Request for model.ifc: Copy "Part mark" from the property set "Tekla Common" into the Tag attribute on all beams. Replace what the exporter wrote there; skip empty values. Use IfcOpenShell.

First a look at what the model holds.

```python
import ifcopenshell
import ifcopenshell.util.element

model = ifcopenshell.open("model.ifc")
print(model.schema)
beams = model.by_type("IfcBeam")
print(len(beams), "beams")
for e in beams[:8]:
    source = ifcopenshell.util.element.get_pset(e, "Tekla Common", "Part mark")
    target = e.Tag
    print(e.id(), repr(source), repr(target), sep=" | ")
```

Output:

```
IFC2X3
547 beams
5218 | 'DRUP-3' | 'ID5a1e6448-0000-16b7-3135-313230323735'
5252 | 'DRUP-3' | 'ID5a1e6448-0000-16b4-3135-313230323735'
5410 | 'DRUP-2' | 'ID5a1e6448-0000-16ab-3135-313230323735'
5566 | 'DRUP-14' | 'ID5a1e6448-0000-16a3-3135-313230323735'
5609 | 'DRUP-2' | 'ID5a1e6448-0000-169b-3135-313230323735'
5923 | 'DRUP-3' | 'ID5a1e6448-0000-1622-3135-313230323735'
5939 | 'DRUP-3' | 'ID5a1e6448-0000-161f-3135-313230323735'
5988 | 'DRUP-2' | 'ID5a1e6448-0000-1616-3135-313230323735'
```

```python
import ifcopenshell
import ifcopenshell.util.element

model = ifcopenshell.open("model.ifc")

count = 0
for e in model.by_type("IfcBeam"):
    value = ifcopenshell.util.element.get_pset(e, "Tekla Common", "Part mark")
    current = e.Tag
    if not value or not value.strip() or current == value:
        continue
    e.Tag = value
    count += 1

print(count, "beams updated")

model.write("model-out.ifc")
```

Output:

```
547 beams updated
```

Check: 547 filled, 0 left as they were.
